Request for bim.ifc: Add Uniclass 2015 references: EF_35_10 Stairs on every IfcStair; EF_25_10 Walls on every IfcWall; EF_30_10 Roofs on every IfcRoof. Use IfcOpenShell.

First a look at what the model holds.

```python
import ifcopenshell

model = ifcopenshell.open("bim.ifc")
print(model.schema)
print("classifications:", [c.Name for c in model.by_type("IfcClassification")])
for ifc_class in ("IfcDoor", "IfcRoof", "IfcStair", "IfcWall", "IfcWindow"):
    print(ifc_class, len(model.by_type(ifc_class)))
```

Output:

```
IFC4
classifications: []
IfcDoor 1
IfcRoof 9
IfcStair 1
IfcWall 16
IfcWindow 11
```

```python
import ifcopenshell
import ifcopenshell.api.classification

model = ifcopenshell.open("bim.ifc")

system = ifcopenshell.api.classification.add_classification(model, classification="Uniclass 2015")

codes = {
    "IfcStair": ("EF_35_10", "Stairs"),
    "IfcWall": ("EF_25_10", "Walls"),
    "IfcRoof": ("EF_30_10", "Roofs"),
}
for ifc_class, (code, name) in codes.items():
    products = model.by_type(ifc_class)
    ifcopenshell.api.classification.add_reference(
        model, products=products, classification=system, identification=code, name=name
    )
    print(code, len(products))

model.write("bim_v2.ifc")
```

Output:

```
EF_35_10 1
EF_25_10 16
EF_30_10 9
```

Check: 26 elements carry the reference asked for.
